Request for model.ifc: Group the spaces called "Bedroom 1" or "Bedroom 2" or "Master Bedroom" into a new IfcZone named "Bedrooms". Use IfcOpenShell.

First a look at what the model holds.

```python
import ifcopenshell

model = ifcopenshell.open("model.ifc")
print(model.schema)
seen = {}
for space in model.by_type("IfcSpace"):
    seen[space.LongName] = seen.get(space.LongName, 0) + 1
for name, count in sorted(seen.items(), key=str):
    print(count, "x", name)
print("zones:", [z.Name for z in model.by_type("IfcZone")][:20])
```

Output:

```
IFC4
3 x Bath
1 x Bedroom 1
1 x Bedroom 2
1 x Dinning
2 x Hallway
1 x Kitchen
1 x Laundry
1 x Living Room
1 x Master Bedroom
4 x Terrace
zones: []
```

```python
import ifcopenshell
import ifcopenshell.api.group
import ifcopenshell.api.root

model = ifcopenshell.open("model.ifc")

names = {"Bedroom 1", "Bedroom 2", "Master Bedroom"}
spaces = [s for s in model.by_type("IfcSpace") if s.LongName in names]

zone = ifcopenshell.api.root.create_entity(model, ifc_class="IfcZone", name="Bedrooms")
ifcopenshell.api.group.assign_group(model, products=spaces, group=zone)
print(len(spaces), "spaces in", zone.Name)

model.write("model-out.ifc")
```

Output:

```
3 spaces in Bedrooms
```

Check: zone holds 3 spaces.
